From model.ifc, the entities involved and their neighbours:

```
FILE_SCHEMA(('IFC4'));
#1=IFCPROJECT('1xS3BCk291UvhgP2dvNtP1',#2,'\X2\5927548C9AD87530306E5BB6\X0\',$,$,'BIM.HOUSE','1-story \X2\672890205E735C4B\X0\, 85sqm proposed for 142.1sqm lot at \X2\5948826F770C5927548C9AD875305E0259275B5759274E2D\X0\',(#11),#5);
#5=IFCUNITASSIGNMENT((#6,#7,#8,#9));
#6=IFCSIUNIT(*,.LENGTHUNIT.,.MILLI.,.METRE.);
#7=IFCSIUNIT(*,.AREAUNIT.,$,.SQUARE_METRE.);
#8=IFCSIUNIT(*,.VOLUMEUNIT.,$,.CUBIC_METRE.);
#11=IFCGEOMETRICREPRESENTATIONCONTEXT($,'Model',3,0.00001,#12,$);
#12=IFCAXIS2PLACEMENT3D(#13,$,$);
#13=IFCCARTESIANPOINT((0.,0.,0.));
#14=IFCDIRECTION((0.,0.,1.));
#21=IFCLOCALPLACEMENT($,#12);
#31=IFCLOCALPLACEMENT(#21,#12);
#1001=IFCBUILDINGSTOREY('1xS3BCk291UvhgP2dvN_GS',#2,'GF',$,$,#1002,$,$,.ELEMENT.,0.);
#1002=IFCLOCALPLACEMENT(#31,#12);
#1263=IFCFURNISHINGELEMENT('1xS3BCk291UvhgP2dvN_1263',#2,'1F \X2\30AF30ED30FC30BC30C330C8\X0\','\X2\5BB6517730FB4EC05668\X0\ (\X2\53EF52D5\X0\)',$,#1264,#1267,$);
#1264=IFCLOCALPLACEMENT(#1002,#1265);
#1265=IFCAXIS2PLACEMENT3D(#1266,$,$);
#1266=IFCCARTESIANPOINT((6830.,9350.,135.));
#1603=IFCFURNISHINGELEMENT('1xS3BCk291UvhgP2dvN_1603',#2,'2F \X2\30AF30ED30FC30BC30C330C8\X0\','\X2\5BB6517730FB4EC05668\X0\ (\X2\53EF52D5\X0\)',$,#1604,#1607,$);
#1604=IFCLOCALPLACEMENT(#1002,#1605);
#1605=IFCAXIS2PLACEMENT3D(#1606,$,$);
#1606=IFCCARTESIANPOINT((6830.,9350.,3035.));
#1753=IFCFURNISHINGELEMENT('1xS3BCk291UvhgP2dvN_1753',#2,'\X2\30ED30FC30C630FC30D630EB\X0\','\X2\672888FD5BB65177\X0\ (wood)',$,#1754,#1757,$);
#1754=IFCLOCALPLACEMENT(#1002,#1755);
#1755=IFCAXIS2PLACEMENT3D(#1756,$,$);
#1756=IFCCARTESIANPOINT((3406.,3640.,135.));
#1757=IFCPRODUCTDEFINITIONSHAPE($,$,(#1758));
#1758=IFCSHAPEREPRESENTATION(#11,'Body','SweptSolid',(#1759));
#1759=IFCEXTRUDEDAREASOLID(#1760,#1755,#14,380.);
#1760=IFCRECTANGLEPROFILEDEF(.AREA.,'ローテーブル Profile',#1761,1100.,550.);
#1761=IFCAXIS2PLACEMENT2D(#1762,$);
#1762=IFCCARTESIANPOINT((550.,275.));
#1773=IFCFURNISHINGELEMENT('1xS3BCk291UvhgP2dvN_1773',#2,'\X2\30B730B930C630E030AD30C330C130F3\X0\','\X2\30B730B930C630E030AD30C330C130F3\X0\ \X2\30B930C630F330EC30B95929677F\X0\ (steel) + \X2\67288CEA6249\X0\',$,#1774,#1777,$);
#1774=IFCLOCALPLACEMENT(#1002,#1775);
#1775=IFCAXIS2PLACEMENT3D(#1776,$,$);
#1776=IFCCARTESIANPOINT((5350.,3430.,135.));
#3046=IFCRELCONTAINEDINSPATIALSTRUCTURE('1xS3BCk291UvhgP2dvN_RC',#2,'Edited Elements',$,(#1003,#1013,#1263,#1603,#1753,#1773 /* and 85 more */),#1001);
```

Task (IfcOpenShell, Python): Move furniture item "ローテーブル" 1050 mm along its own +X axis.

```python
import ifcopenshell
import ifcopenshell.api.geometry
import ifcopenshell.util.placement

model = ifcopenshell.open("model.ifc")

item = model.by_id(1753)
matrix = ifcopenshell.util.placement.get_local_placement(item.ObjectPlacement)
matrix[:3, 3] += matrix[:3, 0] * 1050.0
ifcopenshell.api.geometry.edit_object_placement(model, product=item, matrix=matrix, is_si=False)

print(ifcopenshell.util.placement.get_local_placement(item.ObjectPlacement).round(3) + 0.0)

model.write("model_updated.ifc")
```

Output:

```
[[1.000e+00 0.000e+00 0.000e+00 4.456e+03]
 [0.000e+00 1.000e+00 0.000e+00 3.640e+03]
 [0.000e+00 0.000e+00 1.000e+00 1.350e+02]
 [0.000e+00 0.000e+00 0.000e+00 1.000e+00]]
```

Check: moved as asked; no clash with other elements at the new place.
